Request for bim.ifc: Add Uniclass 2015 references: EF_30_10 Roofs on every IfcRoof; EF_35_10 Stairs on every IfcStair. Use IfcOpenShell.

First a look at what the model holds.

```python
import ifcopenshell

model = ifcopenshell.open("bim.ifc")
print(model.schema)
print("classifications:", [c.Name for c in model.by_type("IfcClassification")])
for ifc_class in ("IfcDoor", "IfcRoof", "IfcStair", "IfcWall", "IfcWindow"):
    print(ifc_class, len(model.by_type(ifc_class)))
```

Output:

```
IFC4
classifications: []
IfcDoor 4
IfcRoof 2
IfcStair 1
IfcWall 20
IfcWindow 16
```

```python
import ifcopenshell
import ifcopenshell.api.classification

model = ifcopenshell.open("bim.ifc")

system = ifcopenshell.api.classification.add_classification(model, classification="Uniclass 2015")

codes = {
    "IfcRoof": ("EF_30_10", "Roofs"),
    "IfcStair": ("EF_35_10", "Stairs"),
}
for ifc_class, (code, name) in codes.items():
    products = model.by_type(ifc_class)
    ifcopenshell.api.classification.add_reference(
        model, products=products, classification=system, identification=code, name=name
    )
    print(code, len(products))

model.write("bim_rev.ifc")
```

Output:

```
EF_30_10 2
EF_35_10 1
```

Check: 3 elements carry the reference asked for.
